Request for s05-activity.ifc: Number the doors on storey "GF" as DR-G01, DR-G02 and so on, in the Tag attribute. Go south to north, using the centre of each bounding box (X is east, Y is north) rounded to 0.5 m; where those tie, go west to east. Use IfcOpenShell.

First a look at what the model holds.

```python
import ifcopenshell
import ifcopenshell.util.element
import ifcopenshell.util.placement

model = ifcopenshell.open("s05-activity.ifc")
print(model.schema)
storey = next(s for s in model.by_type("IfcBuildingStorey") if s.Name == "GF")
doors = [e for e in ifcopenshell.util.element.get_decomposition(storey) if e.is_a("IfcDoor")]
for e in sorted(doors, key=lambda e: e.id()):
    origin = ifcopenshell.util.placement.get_local_placement(e.ObjectPlacement)[:3, 3]
    print(e.id(), e.Tag, e.Name, origin.round(2) + 0.0, sep=" | ")
```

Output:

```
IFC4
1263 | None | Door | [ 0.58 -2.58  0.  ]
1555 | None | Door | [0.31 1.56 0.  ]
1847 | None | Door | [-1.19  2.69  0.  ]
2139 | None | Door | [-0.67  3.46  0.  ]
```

```python
import ifcopenshell
import ifcopenshell.geom
import ifcopenshell.util.element
import ifcopenshell.util.shape

model = ifcopenshell.open("s05-activity.ifc")
settings = ifcopenshell.geom.settings()
settings.set("use-world-coords", True)


def centre(element):
    shape = ifcopenshell.geom.create_shape(settings, element)
    return ifcopenshell.util.shape.get_bbox_centroid(shape.geometry)


storey = next(s for s in model.by_type("IfcBuildingStorey") if s.Name == "GF")
doors = [e for e in ifcopenshell.util.element.get_decomposition(storey) if e.is_a("IfcDoor")]

# Insertion points can sit at a corner or the storey origin, so sort by the geometry (in metres).
centres = {e: centre(e) for e in doors}
doors.sort(key=lambda e: (round(centres[e][1] / 0.5), centres[e][0]))

for i, e in enumerate(doors, start=1):
    number = f"DR-G{i:02d}"
    e.Tag = number
    print(e.id(), number)

model.write("s05-activity-out.ifc")
```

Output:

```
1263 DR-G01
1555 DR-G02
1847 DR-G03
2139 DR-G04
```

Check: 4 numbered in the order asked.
